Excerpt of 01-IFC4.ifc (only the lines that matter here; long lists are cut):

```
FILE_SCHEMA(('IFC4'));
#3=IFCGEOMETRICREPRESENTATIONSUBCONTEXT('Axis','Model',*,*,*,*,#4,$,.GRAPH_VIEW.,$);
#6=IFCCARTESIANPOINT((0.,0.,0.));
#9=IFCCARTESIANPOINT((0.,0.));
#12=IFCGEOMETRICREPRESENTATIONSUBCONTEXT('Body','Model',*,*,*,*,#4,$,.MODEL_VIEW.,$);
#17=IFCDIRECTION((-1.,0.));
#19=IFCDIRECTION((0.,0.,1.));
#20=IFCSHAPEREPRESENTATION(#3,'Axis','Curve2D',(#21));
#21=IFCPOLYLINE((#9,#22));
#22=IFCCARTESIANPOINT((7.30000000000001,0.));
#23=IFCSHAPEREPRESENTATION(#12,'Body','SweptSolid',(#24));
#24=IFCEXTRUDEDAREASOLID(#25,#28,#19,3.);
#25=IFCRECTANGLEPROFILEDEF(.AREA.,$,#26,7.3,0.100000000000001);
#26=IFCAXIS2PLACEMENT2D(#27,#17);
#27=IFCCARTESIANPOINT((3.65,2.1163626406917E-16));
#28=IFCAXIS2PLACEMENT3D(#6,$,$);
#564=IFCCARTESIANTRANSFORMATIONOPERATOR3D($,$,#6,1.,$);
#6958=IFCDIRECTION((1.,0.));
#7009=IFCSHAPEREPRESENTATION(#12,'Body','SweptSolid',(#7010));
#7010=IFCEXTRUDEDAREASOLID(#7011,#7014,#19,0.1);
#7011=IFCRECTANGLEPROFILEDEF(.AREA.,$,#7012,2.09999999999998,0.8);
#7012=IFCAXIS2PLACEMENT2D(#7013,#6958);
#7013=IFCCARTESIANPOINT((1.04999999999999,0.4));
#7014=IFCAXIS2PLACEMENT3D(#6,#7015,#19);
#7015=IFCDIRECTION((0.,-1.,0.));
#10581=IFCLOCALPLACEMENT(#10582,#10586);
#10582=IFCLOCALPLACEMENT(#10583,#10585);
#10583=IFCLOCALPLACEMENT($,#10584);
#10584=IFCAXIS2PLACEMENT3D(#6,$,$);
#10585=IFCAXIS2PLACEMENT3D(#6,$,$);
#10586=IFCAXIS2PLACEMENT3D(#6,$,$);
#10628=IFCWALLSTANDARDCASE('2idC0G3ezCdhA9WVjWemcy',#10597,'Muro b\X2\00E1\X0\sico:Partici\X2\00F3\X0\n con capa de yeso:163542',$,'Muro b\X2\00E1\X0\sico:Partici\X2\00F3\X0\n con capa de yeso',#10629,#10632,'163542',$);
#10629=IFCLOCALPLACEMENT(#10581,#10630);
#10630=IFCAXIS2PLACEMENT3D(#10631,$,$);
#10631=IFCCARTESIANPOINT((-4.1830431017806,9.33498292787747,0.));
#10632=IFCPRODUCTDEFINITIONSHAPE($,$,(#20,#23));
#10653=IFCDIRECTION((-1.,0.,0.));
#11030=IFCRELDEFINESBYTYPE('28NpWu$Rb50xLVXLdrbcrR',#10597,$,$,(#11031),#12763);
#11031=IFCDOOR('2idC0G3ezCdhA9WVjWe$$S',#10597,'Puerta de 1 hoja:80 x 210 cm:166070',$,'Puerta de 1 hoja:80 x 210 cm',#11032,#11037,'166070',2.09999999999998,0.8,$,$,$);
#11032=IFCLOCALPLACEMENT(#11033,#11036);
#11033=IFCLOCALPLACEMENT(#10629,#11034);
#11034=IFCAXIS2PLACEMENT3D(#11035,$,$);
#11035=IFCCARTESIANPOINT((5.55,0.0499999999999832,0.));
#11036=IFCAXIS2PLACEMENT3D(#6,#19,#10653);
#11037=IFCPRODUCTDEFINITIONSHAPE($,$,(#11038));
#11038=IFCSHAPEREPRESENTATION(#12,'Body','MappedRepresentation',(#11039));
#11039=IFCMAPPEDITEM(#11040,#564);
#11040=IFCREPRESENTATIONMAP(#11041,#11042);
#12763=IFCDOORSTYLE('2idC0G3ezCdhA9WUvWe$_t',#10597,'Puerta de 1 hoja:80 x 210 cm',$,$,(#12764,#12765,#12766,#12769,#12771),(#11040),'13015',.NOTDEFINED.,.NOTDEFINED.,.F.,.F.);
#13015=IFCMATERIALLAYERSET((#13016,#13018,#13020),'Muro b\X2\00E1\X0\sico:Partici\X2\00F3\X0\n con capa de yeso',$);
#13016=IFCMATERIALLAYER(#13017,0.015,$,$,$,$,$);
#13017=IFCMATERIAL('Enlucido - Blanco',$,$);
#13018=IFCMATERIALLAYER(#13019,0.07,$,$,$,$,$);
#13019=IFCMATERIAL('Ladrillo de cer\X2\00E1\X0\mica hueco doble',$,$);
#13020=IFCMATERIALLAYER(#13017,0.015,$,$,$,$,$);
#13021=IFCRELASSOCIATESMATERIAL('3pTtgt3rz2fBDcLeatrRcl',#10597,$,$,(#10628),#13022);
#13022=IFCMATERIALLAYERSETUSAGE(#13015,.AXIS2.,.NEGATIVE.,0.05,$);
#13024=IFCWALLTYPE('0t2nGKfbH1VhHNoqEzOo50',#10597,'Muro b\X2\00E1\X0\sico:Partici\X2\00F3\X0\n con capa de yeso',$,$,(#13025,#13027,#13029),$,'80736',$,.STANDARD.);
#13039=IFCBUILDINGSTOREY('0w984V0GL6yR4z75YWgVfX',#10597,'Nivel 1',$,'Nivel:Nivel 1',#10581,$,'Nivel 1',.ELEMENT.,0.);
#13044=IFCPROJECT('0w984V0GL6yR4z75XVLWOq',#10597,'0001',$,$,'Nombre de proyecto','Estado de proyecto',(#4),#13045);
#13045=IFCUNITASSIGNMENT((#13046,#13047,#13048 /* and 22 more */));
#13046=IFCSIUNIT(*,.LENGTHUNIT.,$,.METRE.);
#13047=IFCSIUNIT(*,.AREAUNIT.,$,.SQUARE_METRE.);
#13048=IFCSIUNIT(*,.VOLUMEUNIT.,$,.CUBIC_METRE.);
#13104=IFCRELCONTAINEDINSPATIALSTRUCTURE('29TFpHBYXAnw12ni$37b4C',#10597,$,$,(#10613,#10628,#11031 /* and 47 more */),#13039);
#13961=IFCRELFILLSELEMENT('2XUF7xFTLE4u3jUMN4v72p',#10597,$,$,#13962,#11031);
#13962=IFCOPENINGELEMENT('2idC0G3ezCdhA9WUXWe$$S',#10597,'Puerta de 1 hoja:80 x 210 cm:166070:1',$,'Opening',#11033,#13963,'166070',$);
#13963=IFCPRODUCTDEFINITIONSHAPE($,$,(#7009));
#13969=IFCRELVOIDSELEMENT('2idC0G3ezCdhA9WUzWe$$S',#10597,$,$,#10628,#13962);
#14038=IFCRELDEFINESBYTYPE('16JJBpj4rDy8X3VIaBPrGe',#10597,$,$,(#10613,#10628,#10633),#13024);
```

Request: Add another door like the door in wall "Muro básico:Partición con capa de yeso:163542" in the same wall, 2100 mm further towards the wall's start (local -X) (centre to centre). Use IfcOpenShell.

```python
import ifcopenshell
import ifcopenshell.api.feature
import ifcopenshell.api.geometry
import ifcopenshell.api.root
import ifcopenshell.geom
import ifcopenshell.util.element
import ifcopenshell.util.placement
import ifcopenshell.util.shape
import ifcopenshell.util.unit

model = ifcopenshell.open("01-IFC4.ifc")
unit_scale = ifcopenshell.util.unit.calculate_unit_scale(model)
settings = ifcopenshell.geom.settings()


def volume(element):
    """Net volume in cubic metres, openings subtracted."""
    shape = ifcopenshell.geom.create_shape(settings, element)
    return ifcopenshell.util.shape.get_volume(shape.geometry)


def reuse_history(source, copy):
    """copy_class also copies each property set's owner history, people and application; keep the originals."""
    for rel in copy.IsDefinedBy:
        if rel.is_a("IfcRelDefinesByProperties") and (history := rel.RelatingPropertyDefinition.OwnerHistory):
            rel.RelatingPropertyDefinition.OwnerHistory = source.OwnerHistory
            ifcopenshell.util.element.remove_deep2(model, history)


door = model.by_guid("2idC0G3ezCdhA9WVjWe$$S")
opening = door.FillsVoids[0].RelatingOpeningElement
wall = opening.VoidsElements[0].RelatingBuildingElement
before = volume(wall)
shift = ifcopenshell.util.placement.get_local_placement(wall.ObjectPlacement)[:3, 0] * -2.1 / unit_scale

# copy_class copies the void relationship, type, container and properties, but no geometry.
new_opening = ifcopenshell.api.root.copy_class(model, product=opening)
new_opening.Representation = ifcopenshell.util.element.copy_deep(
    model, opening.Representation, exclude=["IfcGeometricRepresentationContext", "IfcRepresentationMap"]
)
new_opening.Name = "Puerta de 1 hoja:80 x 210 cm"
new_opening.Tag = None
new_door = ifcopenshell.api.root.copy_class(model, product=door)
new_door.Representation = ifcopenshell.util.element.copy_deep(
    model, door.Representation, exclude=["IfcGeometricRepresentationContext", "IfcRepresentationMap"]
)
new_door.Name = "Puerta de 1 hoja:80 x 210 cm"
new_door.Tag = None
reuse_history(door, new_door)
ifcopenshell.api.feature.add_filling(model, opening=new_opening, element=new_door)

for old, new in ((opening, new_opening), (door, new_door)):
    matrix = ifcopenshell.util.placement.get_local_placement(old.ObjectPlacement)
    matrix[:3, 3] += shift
    ifcopenshell.api.geometry.edit_object_placement(model, product=new, matrix=matrix, is_si=False)

after = volume(wall)

print(f"wall volume {before:.3f} -> {after:.3f} m3")

model.write("01-IFC4_v2.ifc")
```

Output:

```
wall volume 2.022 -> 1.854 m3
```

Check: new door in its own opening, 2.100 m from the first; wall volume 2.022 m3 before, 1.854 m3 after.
